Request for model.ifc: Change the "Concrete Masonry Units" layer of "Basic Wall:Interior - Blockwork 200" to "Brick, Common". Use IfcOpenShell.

First a look at what the model holds.

```python
import ifcopenshell
import ifcopenshell.util.element

model = ifcopenshell.open("model.ifc")
print(model.schema)
for layer_set in model.by_type("IfcMaterialLayerSet"):
    if layer_set.LayerSetName == "Basic Wall:Interior - Blockwork 200":
        for layer in layer_set.MaterialLayers:
            print(layer.id(), layer.Material and layer.Material.Name, layer.LayerThickness, sep=" | ")
        print(len(ifcopenshell.util.element.get_elements_by_material(model, layer_set)), "elements and types use it")
print(sorted(m.Name for m in model.by_type("IfcMaterial") if m.Name)[:60])
```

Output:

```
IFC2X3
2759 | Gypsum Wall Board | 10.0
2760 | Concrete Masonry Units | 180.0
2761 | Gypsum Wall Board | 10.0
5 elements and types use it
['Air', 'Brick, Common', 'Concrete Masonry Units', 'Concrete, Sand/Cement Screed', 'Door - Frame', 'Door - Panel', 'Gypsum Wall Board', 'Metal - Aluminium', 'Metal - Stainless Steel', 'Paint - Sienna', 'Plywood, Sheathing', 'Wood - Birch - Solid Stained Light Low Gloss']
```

```python
import ifcopenshell
import ifcopenshell.api.material

model = ifcopenshell.open("model.ifc")

layer_set = next(s for s in model.by_type("IfcMaterialLayerSet") if s.LayerSetName == "Basic Wall:Interior - Blockwork 200")
layer = next(l for l in layer_set.MaterialLayers if l.Material and l.Material.Name == "Concrete Masonry Units")
material = next(m for m in model.by_type("IfcMaterial") if m.Name == "Brick, Common")

# Point this one layer at the other material; renaming the old one would change it everywhere.
ifcopenshell.api.material.edit_layer(model, layer=layer, attributes={}, material=material)

print([l.Material.Name if l.Material else None for l in layer_set.MaterialLayers])

model.write("model_v2.ifc")
```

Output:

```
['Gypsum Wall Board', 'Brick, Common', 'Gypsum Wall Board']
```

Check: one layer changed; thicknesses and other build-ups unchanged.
